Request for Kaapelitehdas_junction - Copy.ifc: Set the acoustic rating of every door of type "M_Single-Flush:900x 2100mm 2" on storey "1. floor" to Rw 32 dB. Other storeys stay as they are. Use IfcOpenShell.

First a look at what the model holds.

```python
import ifcopenshell
import ifcopenshell.util.element

model = ifcopenshell.open("Kaapelitehdas_junction - Copy.ifc")
print(model.schema)
storey = next(s for s in model.by_type("IfcBuildingStorey") if s.Name == "1. floor")
doors = [e for e in ifcopenshell.util.element.get_decomposition(storey) if e.is_a("IfcDoor")]
seen = {}
for e in doors:
    element_type = ifcopenshell.util.element.get_type(e)
    key = (element_type.Name if element_type != e and element_type else None, ifcopenshell.util.element.get_pset(e, "Pset_DoorCommon", "AcousticRating"))
    seen[key] = seen.get(key, 0) + 1
for (name, value), count in sorted(seen.items(), key=str):
    print(count, "x", name, "|", value)
```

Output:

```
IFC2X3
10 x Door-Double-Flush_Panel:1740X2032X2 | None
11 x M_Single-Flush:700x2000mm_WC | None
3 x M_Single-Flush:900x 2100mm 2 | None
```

```python
import ifcopenshell
import ifcopenshell.api.pset
import ifcopenshell.util.element

model = ifcopenshell.open("Kaapelitehdas_junction - Copy.ifc")

storey = next(s for s in model.by_type("IfcBuildingStorey") if s.Name == "1. floor")
doors = [e for e in ifcopenshell.util.element.get_decomposition(storey) if e.is_a("IfcDoor")]

count = 0
for e in doors:
    element_type = ifcopenshell.util.element.get_type(e)
    if element_type in (None, e) or element_type.Name != "M_Single-Flush:900x 2100mm 2":
        continue
    # add_pset returns the element's existing set when there is one.
    pset = ifcopenshell.api.pset.add_pset(model, product=e, name="Pset_DoorCommon")
    ifcopenshell.api.pset.edit_pset(model, pset=pset, properties={"AcousticRating": "Rw 32 dB"})
    count += 1

print(count, "doors updated")

model.write("Kaapelitehdas_junction - Copy-out.ifc")
```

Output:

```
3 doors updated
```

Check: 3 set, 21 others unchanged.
